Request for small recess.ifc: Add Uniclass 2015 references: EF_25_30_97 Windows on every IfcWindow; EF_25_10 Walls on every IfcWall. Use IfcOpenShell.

First a look at what the model holds.

```python
import ifcopenshell

model = ifcopenshell.open("small recess.ifc")
print(model.schema)
print("classifications:", [c.Name for c in model.by_type("IfcClassification")])
for ifc_class in ("IfcDoor", "IfcRoof", "IfcStair", "IfcWall", "IfcWindow"):
    print(ifc_class, len(model.by_type(ifc_class)))
```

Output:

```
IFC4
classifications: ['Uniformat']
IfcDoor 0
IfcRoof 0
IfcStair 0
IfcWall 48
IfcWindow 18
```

```python
import ifcopenshell
import ifcopenshell.api.classification

model = ifcopenshell.open("small recess.ifc")

system = ifcopenshell.api.classification.add_classification(model, classification="Uniclass 2015")

codes = {
    "IfcWindow": ("EF_25_30_97", "Windows"),
    "IfcWall": ("EF_25_10", "Walls"),
}
for ifc_class, (code, name) in codes.items():
    products = model.by_type(ifc_class)
    ifcopenshell.api.classification.add_reference(
        model, products=products, classification=system, identification=code, name=name
    )
    print(code, len(products))

model.write("small recess-out.ifc")
```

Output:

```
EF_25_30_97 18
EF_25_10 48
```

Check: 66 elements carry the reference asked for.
